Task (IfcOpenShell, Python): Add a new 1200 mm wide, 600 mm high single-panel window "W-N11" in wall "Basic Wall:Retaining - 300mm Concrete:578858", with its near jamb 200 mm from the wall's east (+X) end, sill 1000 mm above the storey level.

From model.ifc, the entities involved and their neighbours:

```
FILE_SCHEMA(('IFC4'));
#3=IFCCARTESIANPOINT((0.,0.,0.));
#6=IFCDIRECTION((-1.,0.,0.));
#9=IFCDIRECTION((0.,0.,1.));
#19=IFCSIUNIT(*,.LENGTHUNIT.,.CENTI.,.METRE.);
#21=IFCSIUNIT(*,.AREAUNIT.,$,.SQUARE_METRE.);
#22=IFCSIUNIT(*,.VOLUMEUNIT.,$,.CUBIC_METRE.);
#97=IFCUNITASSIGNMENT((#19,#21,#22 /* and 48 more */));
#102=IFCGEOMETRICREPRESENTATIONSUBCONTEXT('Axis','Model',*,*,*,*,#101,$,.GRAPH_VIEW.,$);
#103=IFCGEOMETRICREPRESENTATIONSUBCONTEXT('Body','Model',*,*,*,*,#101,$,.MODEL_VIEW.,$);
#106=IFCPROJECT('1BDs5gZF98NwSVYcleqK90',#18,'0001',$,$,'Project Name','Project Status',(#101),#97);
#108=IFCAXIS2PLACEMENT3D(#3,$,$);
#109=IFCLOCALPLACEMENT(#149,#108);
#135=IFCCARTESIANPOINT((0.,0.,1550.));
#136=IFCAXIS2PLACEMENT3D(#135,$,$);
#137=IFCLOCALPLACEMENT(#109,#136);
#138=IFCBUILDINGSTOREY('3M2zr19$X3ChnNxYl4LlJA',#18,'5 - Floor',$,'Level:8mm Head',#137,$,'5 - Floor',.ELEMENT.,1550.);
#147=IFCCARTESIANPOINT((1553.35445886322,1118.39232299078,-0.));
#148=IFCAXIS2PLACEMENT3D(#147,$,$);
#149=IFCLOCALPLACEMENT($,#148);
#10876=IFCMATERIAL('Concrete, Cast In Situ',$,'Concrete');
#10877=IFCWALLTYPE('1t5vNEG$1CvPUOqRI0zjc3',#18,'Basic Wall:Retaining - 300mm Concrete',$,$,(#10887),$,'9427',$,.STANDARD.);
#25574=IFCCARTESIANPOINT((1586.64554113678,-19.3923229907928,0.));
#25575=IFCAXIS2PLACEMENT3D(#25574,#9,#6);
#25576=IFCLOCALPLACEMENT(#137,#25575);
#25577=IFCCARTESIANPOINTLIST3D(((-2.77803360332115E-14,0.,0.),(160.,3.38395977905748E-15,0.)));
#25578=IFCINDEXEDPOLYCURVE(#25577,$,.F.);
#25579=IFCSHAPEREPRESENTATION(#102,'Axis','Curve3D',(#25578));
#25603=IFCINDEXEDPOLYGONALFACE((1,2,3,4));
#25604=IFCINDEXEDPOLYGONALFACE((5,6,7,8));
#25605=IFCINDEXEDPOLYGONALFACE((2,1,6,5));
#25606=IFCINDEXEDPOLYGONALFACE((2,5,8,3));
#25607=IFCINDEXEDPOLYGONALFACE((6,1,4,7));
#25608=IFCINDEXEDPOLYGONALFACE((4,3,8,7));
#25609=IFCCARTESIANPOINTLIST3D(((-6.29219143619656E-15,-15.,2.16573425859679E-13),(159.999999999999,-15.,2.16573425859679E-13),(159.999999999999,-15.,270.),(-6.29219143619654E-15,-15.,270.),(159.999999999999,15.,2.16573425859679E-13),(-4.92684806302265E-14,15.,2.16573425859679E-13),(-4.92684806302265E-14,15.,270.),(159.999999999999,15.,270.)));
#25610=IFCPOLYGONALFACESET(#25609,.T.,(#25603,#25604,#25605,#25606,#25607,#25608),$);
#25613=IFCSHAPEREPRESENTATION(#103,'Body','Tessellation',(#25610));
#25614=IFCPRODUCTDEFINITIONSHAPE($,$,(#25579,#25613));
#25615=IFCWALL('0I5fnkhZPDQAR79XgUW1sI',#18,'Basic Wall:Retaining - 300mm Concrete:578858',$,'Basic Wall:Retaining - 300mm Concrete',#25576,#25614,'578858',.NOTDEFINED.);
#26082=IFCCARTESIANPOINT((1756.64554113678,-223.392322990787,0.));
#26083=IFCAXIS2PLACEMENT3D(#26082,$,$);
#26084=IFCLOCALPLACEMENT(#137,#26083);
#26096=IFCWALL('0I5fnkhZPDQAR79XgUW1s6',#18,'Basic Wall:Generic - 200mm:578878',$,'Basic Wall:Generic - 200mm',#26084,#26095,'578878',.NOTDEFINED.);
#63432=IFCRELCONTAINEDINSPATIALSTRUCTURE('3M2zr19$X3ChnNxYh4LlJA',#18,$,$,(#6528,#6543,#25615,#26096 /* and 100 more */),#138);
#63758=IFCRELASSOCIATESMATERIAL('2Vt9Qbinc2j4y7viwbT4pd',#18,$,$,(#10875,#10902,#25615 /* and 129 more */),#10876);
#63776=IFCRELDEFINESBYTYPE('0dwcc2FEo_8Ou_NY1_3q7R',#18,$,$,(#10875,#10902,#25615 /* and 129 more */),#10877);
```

```python
import numpy as np
import ifcopenshell
import ifcopenshell.api.feature
import ifcopenshell.api.geometry
import ifcopenshell.api.root
import ifcopenshell.api.spatial
import ifcopenshell.geom
import ifcopenshell.util.element
import ifcopenshell.util.placement
import ifcopenshell.util.representation
import ifcopenshell.util.shape
import ifcopenshell.util.unit

model = ifcopenshell.open("model.ifc")
unit_scale = ifcopenshell.util.unit.calculate_unit_scale(model)
settings = ifcopenshell.geom.settings()


def volume(element):
    """Net volume in cubic metres, openings subtracted."""
    shape = ifcopenshell.geom.create_shape(settings, element)
    return ifcopenshell.util.shape.get_volume(shape.geometry)


wall = model.by_guid("0I5fnkhZPDQAR79XgUW1sI")
storey = ifcopenshell.util.element.get_container(wall, ifc_class="IfcBuildingStorey")
context = ifcopenshell.util.representation.get_context(model, "Model", "Body", "MODEL_VIEW")
before = volume(wall)

width, height, from_end, sill = 1.2, 0.6, 0.2, 1  # metres

# The wall runs along its own X axis, and the end named is its -X end.
wall_shape = ifcopenshell.geom.create_shape(settings, wall)
x, y, z = ifcopenshell.util.shape.get_vertices(wall_shape.geometry).T
start = x.min() + from_end
face, thickness = float(y.min()), float(y.max() - y.min())
wall_matrix = ifcopenshell.util.placement.get_local_placement(wall.ObjectPlacement)
level = ifcopenshell.util.placement.get_local_placement(storey.ObjectPlacement)[2, 3]


def in_wall(x, y):
    """Placement at x, y metres in the wall's axes, at sill height."""
    matrix = wall_matrix.copy()
    matrix[:, 3] = wall_matrix @ np.array([x / unit_scale, y / unit_scale, 0.0, 1.0])
    matrix[2, 3] = level + sill / unit_scale
    return matrix


# Opening: a box that overshoots both wall faces by 50 mm.
opening = ifcopenshell.api.root.create_entity(model, ifc_class="IfcOpeningElement", predefined_type="OPENING")
box = ifcopenshell.api.geometry.add_wall_representation(
    model, context=context, length=width, height=height, thickness=thickness + 0.1
)
ifcopenshell.api.geometry.assign_representation(model, product=opening, representation=box)
ifcopenshell.api.geometry.edit_object_placement(model, product=opening, matrix=in_wall(start, face - 0.05), is_si=False)
ifcopenshell.api.feature.add_feature(model, feature=opening, element=wall)

window = ifcopenshell.api.root.create_entity(model, ifc_class="IfcWindow", name="W-N11", predefined_type="WINDOW")
window.OverallWidth, window.OverallHeight = width / unit_scale, height / unit_scale
window.PartitioningType = "SINGLE_PANEL"
body = ifcopenshell.api.geometry.add_window_representation(
    model,
    context=context,
    overall_width=window.OverallWidth,
    overall_height=window.OverallHeight,
    partition_type="SINGLE_PANEL",
)
ifcopenshell.api.geometry.assign_representation(model, product=window, representation=body)
ifcopenshell.api.spatial.assign_container(model, products=[window], relating_structure=storey)
ifcopenshell.api.feature.add_filling(model, opening=opening, element=window)

# Centre the window in the wall's thickness.
ifcopenshell.api.geometry.edit_object_placement(model, product=window, matrix=in_wall(start, face), is_si=False)
window_shape = ifcopenshell.geom.create_shape(settings, window)
depth = ifcopenshell.util.shape.get_vertices(window_shape.geometry)[:, 1]
offset = face + thickness / 2 - (depth.min() + depth.max()) / 2
ifcopenshell.api.geometry.edit_object_placement(model, product=window, matrix=in_wall(start, offset), is_si=False)

after = volume(wall)

print(f"wall volume {before:.3f} -> {after:.3f} m3")

model.write("model_rev.ifc")
```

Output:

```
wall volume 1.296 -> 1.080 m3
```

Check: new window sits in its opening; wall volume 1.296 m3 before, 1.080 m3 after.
